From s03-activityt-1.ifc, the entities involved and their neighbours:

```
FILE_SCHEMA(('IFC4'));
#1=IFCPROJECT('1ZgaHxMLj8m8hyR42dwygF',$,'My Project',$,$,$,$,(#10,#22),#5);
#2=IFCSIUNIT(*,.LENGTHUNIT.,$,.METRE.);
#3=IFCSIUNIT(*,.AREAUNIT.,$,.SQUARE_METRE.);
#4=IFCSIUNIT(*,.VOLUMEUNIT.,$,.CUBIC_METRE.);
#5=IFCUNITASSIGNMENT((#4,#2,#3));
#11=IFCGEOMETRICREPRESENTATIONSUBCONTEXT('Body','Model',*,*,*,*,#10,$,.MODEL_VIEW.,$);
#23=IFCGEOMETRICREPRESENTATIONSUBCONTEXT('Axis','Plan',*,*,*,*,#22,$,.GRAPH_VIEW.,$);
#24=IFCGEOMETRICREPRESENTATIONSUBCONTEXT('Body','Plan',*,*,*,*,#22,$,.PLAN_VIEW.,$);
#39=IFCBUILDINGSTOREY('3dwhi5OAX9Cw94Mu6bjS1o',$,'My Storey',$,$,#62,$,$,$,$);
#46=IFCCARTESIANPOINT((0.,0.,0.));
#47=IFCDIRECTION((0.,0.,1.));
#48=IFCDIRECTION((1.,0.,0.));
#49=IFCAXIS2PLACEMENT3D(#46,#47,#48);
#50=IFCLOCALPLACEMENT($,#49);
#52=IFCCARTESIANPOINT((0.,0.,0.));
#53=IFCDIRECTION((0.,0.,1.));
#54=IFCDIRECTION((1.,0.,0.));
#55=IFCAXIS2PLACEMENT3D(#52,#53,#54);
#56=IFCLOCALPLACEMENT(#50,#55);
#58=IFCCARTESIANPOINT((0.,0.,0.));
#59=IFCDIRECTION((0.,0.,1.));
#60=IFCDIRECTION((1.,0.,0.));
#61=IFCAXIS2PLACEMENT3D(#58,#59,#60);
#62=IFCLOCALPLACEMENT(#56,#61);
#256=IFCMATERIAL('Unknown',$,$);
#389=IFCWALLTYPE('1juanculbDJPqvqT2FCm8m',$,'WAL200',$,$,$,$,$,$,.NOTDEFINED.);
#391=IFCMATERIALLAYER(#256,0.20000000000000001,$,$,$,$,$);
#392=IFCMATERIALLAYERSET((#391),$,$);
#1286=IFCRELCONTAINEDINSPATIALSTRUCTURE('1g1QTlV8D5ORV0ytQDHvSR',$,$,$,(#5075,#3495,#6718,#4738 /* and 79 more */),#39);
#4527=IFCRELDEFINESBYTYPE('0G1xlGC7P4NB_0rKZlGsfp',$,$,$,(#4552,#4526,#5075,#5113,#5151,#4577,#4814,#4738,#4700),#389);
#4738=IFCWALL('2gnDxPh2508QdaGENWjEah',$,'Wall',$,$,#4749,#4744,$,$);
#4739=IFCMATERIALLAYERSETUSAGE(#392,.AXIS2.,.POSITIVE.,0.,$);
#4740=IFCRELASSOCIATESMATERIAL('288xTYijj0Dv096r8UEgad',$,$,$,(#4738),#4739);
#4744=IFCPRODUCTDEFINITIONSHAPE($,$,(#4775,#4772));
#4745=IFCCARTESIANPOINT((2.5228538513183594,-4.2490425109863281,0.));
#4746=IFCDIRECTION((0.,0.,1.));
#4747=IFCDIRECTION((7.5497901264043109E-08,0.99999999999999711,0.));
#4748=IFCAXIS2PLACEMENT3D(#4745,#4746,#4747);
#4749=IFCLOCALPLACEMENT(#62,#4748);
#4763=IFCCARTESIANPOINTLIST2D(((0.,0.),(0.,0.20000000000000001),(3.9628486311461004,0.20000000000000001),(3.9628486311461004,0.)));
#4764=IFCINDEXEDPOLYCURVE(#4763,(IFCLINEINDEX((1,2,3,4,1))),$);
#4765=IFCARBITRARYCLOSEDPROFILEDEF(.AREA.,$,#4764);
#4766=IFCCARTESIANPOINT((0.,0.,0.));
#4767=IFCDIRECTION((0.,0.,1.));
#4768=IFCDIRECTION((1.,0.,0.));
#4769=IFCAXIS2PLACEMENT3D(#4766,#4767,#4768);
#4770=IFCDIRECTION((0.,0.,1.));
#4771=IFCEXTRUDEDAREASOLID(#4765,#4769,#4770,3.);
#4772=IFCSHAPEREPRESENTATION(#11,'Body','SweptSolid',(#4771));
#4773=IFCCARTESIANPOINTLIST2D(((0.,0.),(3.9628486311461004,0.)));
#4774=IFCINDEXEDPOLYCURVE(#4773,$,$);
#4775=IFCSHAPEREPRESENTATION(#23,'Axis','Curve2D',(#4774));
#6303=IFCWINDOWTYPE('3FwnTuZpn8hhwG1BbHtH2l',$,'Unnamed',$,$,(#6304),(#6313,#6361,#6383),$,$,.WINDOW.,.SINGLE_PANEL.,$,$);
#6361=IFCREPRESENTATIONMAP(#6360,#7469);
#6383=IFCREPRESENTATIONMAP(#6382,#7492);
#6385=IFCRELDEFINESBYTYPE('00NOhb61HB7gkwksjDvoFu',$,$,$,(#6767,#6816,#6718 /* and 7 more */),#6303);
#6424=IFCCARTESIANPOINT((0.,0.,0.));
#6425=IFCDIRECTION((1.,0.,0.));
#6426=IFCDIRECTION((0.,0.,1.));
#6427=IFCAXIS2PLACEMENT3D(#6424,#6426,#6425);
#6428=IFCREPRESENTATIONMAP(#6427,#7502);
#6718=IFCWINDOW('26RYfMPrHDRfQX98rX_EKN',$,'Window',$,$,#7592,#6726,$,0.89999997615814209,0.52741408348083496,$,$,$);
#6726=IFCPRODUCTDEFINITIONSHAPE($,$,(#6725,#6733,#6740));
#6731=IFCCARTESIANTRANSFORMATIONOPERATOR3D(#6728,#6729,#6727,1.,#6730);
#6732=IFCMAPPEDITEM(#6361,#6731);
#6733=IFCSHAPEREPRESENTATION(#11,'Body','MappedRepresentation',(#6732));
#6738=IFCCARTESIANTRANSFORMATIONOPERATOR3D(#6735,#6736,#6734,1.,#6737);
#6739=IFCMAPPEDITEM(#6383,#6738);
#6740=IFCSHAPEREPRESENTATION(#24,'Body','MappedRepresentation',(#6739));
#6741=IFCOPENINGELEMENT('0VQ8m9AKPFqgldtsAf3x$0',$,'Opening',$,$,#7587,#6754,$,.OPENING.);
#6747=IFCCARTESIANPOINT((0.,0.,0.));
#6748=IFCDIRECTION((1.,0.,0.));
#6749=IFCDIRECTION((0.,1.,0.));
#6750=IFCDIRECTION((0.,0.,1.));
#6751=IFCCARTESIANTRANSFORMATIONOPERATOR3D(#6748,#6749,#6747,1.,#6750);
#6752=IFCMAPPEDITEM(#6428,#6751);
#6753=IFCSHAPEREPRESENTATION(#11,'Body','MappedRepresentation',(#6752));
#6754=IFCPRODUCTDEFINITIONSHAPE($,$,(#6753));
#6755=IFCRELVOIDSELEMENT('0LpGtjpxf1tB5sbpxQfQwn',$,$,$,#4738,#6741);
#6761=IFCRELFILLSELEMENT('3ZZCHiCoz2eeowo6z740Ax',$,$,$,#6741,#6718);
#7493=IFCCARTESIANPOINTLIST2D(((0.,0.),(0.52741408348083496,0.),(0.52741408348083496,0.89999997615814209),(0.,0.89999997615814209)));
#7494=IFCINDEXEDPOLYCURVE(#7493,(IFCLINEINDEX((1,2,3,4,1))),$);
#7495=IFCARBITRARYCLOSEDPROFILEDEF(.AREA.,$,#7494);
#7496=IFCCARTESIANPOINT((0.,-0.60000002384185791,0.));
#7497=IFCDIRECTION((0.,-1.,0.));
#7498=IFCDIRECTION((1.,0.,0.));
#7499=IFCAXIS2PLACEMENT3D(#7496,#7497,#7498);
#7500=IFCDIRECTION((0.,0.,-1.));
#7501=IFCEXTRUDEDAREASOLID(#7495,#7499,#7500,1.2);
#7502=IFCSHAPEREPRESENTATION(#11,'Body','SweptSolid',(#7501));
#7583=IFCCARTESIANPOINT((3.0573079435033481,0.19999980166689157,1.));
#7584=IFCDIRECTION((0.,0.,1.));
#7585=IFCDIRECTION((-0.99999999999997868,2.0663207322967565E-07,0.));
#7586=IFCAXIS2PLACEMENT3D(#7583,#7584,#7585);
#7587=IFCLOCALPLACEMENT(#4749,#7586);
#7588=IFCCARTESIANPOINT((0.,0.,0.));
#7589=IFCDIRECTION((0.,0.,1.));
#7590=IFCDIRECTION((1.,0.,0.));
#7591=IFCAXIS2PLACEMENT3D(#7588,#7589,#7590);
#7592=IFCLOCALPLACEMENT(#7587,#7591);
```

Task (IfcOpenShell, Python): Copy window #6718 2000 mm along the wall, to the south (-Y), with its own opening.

```python
import ifcopenshell
import ifcopenshell.api.feature
import ifcopenshell.api.geometry
import ifcopenshell.api.root
import ifcopenshell.geom
import ifcopenshell.util.element
import ifcopenshell.util.placement
import ifcopenshell.util.shape
import ifcopenshell.util.unit

model = ifcopenshell.open("s03-activityt-1.ifc")
unit_scale = ifcopenshell.util.unit.calculate_unit_scale(model)
settings = ifcopenshell.geom.settings()


def volume(element):
    """Net volume in cubic metres, openings subtracted."""
    shape = ifcopenshell.geom.create_shape(settings, element)
    return ifcopenshell.util.shape.get_volume(shape.geometry)


window = model.by_id(6718)
opening = window.FillsVoids[0].RelatingOpeningElement
wall = opening.VoidsElements[0].RelatingBuildingElement
before = volume(wall)
shift = ifcopenshell.util.placement.get_local_placement(wall.ObjectPlacement)[:3, 0] * -2 / unit_scale

# copy_class copies the void relationship, type, container and properties, but no geometry.
new_opening = ifcopenshell.api.root.copy_class(model, product=opening)
new_opening.Representation = ifcopenshell.util.element.copy_deep(
    model, opening.Representation, exclude=["IfcGeometricRepresentationContext", "IfcRepresentationMap"]
)
new_window = ifcopenshell.api.root.copy_class(model, product=window)
new_window.Representation = ifcopenshell.util.element.copy_deep(
    model, window.Representation, exclude=["IfcGeometricRepresentationContext", "IfcRepresentationMap"]
)
ifcopenshell.api.feature.add_filling(model, opening=new_opening, element=new_window)

for old, new in ((opening, new_opening), (window, new_window)):
    matrix = ifcopenshell.util.placement.get_local_placement(old.ObjectPlacement)
    matrix[:3, 3] += shift
    ifcopenshell.api.geometry.edit_object_placement(model, product=new, matrix=matrix, is_si=False)

after = volume(wall)

print(f"wall volume {before:.3f} -> {after:.3f} m3")

model.write("s03-activityt-1_rev.ifc")
```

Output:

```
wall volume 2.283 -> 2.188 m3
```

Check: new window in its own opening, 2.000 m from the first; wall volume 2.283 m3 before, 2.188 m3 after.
